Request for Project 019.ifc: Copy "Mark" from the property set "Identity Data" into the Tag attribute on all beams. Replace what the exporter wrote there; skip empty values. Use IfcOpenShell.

First a look at what the model holds.

```python
import ifcopenshell
import ifcopenshell.util.element

model = ifcopenshell.open("Project 019.ifc")
print(model.schema)
beams = model.by_type("IfcBeam")
print(len(beams), "beams")
for e in beams[:8]:
    source = ifcopenshell.util.element.get_pset(e, "Identity Data", "Mark")
    target = e.Tag
    print(e.id(), repr(source), repr(target), sep=" | ")
```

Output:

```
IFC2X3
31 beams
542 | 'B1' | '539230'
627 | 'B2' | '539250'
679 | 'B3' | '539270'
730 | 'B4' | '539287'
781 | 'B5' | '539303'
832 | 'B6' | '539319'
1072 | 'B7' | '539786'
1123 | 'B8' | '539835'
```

```python
import ifcopenshell
import ifcopenshell.util.element

model = ifcopenshell.open("Project 019.ifc")

count = 0
for e in model.by_type("IfcBeam"):
    value = ifcopenshell.util.element.get_pset(e, "Identity Data", "Mark")
    current = e.Tag
    if not value or not value.strip() or current == value:
        continue
    e.Tag = value
    count += 1

print(count, "beams updated")

model.write("Project 019_edited.ifc")
```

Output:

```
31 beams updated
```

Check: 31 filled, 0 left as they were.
